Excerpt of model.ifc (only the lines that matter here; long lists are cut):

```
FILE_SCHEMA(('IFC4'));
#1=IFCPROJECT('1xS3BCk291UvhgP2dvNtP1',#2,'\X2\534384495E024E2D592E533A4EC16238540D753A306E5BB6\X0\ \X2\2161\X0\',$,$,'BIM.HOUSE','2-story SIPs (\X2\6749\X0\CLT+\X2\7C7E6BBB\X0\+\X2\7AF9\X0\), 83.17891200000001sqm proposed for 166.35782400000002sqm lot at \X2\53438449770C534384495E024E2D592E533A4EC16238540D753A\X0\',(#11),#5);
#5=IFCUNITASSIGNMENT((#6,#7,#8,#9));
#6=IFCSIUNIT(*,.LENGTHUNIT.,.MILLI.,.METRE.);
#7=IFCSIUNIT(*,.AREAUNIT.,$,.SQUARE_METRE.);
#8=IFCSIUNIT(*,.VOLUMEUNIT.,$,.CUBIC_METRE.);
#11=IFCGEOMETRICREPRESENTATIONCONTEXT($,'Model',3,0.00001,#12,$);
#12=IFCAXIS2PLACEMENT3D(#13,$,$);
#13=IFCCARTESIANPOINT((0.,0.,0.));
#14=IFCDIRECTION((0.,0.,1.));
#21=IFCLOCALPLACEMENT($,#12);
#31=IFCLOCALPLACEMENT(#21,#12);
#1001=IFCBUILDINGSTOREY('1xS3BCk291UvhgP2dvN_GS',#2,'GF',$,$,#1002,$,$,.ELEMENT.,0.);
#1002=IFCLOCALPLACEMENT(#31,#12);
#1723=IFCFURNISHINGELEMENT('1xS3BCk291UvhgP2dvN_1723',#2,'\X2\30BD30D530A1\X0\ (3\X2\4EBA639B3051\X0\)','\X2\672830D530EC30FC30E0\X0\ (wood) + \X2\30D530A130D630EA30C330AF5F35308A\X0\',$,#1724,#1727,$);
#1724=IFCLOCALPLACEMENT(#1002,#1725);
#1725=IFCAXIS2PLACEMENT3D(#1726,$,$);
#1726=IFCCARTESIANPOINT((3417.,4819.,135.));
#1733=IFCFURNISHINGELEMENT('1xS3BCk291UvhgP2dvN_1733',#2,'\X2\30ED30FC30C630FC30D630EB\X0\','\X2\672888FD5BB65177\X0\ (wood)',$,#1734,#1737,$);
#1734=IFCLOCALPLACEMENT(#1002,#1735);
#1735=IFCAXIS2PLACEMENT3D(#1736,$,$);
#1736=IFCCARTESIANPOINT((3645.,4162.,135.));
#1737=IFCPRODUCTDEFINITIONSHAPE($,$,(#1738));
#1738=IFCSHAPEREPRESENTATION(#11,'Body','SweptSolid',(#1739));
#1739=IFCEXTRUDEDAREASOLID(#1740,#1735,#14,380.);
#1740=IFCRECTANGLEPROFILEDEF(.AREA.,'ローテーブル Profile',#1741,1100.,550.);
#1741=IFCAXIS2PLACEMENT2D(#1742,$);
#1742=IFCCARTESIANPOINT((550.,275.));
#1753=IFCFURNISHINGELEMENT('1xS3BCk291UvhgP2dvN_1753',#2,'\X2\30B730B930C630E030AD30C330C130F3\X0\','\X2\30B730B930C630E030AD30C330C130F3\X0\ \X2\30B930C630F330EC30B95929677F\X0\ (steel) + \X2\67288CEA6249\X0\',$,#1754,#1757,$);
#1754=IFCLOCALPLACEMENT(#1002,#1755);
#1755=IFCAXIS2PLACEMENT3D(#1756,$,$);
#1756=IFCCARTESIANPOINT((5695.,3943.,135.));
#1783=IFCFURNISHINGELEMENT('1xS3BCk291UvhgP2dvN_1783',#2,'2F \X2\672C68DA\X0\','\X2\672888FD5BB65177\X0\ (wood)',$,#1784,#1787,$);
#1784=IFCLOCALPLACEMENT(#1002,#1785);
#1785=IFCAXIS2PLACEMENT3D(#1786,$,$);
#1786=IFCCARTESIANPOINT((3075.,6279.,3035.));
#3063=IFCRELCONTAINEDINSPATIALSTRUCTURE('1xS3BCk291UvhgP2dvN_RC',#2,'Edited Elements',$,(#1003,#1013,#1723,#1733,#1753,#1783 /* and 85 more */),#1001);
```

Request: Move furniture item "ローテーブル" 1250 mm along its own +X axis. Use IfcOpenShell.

```python
import ifcopenshell
import ifcopenshell.api.geometry
import ifcopenshell.util.placement

model = ifcopenshell.open("model.ifc")

item = model.by_guid("1xS3BCk291UvhgP2dvN_1733")
matrix = ifcopenshell.util.placement.get_local_placement(item.ObjectPlacement)
matrix[:3, 3] += matrix[:3, 0] * 1250.0
ifcopenshell.api.geometry.edit_object_placement(model, product=item, matrix=matrix, is_si=False)

print(ifcopenshell.util.placement.get_local_placement(item.ObjectPlacement).round(3) + 0.0)

model.write("model_updated.ifc")
```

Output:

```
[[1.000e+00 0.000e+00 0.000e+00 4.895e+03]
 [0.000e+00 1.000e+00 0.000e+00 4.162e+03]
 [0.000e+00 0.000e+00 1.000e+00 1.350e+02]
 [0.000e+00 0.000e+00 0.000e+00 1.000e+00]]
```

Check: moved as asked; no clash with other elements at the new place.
